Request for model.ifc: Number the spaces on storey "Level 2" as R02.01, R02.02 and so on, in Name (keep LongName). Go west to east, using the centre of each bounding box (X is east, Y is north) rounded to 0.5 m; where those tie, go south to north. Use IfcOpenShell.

First a look at what the model holds.

```python
import ifcopenshell
import ifcopenshell.util.element
import ifcopenshell.util.placement

model = ifcopenshell.open("model.ifc")
print(model.schema)
storey = next(s for s in model.by_type("IfcBuildingStorey") if s.Name == "Level 2")
spaces = [e for e in ifcopenshell.util.element.get_decomposition(storey) if e.is_a("IfcSpace")]
for e in sorted(spaces, key=lambda e: e.id()):
    origin = ifcopenshell.util.placement.get_local_placement(e.ObjectPlacement)[:3, 3]
    print(e.id(), e.Name, e.LongName, origin.round(2) + 0.0, sep=" | ")
```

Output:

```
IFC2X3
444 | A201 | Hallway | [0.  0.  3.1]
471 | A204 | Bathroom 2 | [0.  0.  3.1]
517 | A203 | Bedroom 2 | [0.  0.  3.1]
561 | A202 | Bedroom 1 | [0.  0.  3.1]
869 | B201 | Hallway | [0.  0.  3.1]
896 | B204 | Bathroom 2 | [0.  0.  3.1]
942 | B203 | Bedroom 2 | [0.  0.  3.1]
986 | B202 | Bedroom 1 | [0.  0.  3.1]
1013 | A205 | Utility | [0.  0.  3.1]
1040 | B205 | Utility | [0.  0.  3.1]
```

```python
import ifcopenshell
import ifcopenshell.geom
import ifcopenshell.util.element
import ifcopenshell.util.shape

model = ifcopenshell.open("model.ifc")
settings = ifcopenshell.geom.settings()
settings.set("use-world-coords", True)


def centre(element):
    shape = ifcopenshell.geom.create_shape(settings, element)
    return ifcopenshell.util.shape.get_bbox_centroid(shape.geometry)


storey = next(s for s in model.by_type("IfcBuildingStorey") if s.Name == "Level 2")
spaces = [e for e in ifcopenshell.util.element.get_decomposition(storey) if e.is_a("IfcSpace")]

# Insertion points can sit at a corner or the storey origin, so sort by the geometry (in metres).
centres = {e: centre(e) for e in spaces}
spaces.sort(key=lambda e: (round(centres[e][0] / 0.5), centres[e][1]))

for i, e in enumerate(spaces, start=1):
    number = f"R02.{i:02d}"
    e.Name = number
    print(e.id(), number)

model.write("model_rev.ifc")
```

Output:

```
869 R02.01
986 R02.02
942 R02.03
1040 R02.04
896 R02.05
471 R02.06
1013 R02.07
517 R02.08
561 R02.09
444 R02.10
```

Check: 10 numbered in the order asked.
